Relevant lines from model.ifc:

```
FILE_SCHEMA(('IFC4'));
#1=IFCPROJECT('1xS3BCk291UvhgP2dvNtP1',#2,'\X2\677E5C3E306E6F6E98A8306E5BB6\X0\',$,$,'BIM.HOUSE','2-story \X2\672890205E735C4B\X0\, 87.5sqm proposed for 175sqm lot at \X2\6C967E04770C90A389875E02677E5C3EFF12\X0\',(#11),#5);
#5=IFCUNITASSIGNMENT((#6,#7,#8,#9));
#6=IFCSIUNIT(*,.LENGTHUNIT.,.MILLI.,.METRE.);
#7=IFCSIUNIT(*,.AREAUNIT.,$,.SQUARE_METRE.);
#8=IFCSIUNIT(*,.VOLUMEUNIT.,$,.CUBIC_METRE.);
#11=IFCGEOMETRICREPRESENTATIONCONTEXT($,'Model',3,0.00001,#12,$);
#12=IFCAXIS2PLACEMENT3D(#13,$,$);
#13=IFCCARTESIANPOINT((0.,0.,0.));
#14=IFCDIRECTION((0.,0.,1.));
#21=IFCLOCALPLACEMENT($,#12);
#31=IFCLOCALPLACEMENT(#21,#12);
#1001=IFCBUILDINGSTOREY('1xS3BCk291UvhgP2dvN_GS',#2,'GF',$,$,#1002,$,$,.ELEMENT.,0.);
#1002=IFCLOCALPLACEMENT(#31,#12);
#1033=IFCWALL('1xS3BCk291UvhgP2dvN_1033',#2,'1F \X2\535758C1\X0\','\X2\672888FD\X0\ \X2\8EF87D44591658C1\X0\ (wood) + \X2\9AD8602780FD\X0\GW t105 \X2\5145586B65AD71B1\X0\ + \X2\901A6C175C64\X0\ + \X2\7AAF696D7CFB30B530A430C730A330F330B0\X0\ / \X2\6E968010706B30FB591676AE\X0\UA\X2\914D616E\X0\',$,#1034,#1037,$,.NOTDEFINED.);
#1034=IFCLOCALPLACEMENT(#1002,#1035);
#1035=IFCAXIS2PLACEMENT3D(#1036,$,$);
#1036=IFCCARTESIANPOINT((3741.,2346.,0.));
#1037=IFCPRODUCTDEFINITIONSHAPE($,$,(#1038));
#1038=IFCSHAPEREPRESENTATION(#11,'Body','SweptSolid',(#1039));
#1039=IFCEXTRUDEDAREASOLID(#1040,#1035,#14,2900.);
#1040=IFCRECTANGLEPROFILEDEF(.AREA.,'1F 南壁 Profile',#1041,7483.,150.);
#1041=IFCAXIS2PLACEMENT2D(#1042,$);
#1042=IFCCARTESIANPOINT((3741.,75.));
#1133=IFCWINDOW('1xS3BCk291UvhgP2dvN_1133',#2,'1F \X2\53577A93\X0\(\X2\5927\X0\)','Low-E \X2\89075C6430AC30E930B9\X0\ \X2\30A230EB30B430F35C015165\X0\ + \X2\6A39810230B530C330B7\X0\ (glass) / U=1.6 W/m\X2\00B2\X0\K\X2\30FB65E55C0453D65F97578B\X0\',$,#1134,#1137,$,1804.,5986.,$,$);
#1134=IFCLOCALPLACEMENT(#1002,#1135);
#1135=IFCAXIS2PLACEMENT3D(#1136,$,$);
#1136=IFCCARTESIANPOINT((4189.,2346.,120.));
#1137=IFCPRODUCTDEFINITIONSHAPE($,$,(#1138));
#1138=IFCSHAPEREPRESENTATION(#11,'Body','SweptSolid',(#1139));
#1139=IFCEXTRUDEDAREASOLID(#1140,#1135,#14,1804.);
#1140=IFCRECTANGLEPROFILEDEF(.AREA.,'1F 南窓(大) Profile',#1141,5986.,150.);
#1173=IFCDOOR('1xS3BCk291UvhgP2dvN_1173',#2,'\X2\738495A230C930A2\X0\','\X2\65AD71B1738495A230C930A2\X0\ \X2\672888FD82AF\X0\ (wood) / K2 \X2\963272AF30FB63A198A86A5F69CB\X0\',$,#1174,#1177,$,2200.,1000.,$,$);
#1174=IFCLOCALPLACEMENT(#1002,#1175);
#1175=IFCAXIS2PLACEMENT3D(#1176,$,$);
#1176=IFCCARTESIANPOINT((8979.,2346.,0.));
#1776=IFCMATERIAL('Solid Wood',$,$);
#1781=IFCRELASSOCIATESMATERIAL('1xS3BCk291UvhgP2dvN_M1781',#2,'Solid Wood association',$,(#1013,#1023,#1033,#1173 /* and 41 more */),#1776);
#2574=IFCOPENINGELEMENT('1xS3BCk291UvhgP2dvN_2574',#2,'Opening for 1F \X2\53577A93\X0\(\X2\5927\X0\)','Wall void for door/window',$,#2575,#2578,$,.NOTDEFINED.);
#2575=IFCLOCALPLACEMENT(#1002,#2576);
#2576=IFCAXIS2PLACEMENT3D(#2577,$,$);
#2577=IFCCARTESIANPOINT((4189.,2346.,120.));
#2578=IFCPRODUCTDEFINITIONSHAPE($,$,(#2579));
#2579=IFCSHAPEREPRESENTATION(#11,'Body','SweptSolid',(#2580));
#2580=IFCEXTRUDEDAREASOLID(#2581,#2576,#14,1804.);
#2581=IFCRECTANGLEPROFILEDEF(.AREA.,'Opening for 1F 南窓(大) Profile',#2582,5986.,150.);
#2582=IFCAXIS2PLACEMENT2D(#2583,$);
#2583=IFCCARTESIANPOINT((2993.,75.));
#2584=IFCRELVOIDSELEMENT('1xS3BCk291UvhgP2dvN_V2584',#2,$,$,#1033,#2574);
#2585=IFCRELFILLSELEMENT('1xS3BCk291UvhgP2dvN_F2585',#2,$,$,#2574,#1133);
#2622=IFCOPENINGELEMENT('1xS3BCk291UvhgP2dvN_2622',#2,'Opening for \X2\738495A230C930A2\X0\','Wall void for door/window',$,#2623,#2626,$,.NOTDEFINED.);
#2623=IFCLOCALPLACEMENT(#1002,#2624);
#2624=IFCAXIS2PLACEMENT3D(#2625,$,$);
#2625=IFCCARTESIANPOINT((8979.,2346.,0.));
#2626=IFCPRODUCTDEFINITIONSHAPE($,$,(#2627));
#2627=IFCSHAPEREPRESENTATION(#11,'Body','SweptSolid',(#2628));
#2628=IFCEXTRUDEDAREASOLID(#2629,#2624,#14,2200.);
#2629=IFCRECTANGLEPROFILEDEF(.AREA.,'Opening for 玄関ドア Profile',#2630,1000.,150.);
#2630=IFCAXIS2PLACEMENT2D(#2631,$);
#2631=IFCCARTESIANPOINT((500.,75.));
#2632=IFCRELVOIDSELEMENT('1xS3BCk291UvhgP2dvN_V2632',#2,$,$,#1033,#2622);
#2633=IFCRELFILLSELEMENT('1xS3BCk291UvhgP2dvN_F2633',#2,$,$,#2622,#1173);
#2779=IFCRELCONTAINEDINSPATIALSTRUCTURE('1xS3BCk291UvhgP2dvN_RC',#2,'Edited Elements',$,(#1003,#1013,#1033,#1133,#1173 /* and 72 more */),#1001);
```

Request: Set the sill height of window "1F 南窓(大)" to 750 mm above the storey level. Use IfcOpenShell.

```python
import numpy as np
import ifcopenshell
import ifcopenshell.api.geometry
import ifcopenshell.geom
import ifcopenshell.util.element
import ifcopenshell.util.placement
import ifcopenshell.util.shape
import ifcopenshell.util.unit

model = ifcopenshell.open("model.ifc")
unit_scale = ifcopenshell.util.unit.calculate_unit_scale(model)

window = model.by_id(1133)
opening = window.FillsVoids[0].RelatingOpeningElement
storey = ifcopenshell.util.element.get_container(window, ifc_class="IfcBuildingStorey")
level = ifcopenshell.util.placement.get_local_placement(storey.ObjectPlacement)[2, 3]

# The opening's origin need not be at the sill, so measure its lowest point.
shape = ifcopenshell.geom.create_shape(ifcopenshell.geom.settings(), opening)
bottom = ifcopenshell.util.shape.get_shape_bottom_elevation(shape, shape.geometry) / unit_scale
dz = level + 750.0 - bottom

shift = np.array([0.0, 0.0, dz])
# The window is not placed relative to its opening, so move both.
for product in (opening, window):
    matrix = ifcopenshell.util.placement.get_local_placement(product.ObjectPlacement)
    matrix[:3, 3] += shift
    ifcopenshell.api.geometry.edit_object_placement(model, product=product, matrix=matrix, is_si=False)

print(f"moved by {dz * unit_scale:+.3f} m")

model.write("model_edited.ifc")
```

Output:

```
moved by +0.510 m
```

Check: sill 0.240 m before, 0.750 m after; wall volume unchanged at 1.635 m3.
